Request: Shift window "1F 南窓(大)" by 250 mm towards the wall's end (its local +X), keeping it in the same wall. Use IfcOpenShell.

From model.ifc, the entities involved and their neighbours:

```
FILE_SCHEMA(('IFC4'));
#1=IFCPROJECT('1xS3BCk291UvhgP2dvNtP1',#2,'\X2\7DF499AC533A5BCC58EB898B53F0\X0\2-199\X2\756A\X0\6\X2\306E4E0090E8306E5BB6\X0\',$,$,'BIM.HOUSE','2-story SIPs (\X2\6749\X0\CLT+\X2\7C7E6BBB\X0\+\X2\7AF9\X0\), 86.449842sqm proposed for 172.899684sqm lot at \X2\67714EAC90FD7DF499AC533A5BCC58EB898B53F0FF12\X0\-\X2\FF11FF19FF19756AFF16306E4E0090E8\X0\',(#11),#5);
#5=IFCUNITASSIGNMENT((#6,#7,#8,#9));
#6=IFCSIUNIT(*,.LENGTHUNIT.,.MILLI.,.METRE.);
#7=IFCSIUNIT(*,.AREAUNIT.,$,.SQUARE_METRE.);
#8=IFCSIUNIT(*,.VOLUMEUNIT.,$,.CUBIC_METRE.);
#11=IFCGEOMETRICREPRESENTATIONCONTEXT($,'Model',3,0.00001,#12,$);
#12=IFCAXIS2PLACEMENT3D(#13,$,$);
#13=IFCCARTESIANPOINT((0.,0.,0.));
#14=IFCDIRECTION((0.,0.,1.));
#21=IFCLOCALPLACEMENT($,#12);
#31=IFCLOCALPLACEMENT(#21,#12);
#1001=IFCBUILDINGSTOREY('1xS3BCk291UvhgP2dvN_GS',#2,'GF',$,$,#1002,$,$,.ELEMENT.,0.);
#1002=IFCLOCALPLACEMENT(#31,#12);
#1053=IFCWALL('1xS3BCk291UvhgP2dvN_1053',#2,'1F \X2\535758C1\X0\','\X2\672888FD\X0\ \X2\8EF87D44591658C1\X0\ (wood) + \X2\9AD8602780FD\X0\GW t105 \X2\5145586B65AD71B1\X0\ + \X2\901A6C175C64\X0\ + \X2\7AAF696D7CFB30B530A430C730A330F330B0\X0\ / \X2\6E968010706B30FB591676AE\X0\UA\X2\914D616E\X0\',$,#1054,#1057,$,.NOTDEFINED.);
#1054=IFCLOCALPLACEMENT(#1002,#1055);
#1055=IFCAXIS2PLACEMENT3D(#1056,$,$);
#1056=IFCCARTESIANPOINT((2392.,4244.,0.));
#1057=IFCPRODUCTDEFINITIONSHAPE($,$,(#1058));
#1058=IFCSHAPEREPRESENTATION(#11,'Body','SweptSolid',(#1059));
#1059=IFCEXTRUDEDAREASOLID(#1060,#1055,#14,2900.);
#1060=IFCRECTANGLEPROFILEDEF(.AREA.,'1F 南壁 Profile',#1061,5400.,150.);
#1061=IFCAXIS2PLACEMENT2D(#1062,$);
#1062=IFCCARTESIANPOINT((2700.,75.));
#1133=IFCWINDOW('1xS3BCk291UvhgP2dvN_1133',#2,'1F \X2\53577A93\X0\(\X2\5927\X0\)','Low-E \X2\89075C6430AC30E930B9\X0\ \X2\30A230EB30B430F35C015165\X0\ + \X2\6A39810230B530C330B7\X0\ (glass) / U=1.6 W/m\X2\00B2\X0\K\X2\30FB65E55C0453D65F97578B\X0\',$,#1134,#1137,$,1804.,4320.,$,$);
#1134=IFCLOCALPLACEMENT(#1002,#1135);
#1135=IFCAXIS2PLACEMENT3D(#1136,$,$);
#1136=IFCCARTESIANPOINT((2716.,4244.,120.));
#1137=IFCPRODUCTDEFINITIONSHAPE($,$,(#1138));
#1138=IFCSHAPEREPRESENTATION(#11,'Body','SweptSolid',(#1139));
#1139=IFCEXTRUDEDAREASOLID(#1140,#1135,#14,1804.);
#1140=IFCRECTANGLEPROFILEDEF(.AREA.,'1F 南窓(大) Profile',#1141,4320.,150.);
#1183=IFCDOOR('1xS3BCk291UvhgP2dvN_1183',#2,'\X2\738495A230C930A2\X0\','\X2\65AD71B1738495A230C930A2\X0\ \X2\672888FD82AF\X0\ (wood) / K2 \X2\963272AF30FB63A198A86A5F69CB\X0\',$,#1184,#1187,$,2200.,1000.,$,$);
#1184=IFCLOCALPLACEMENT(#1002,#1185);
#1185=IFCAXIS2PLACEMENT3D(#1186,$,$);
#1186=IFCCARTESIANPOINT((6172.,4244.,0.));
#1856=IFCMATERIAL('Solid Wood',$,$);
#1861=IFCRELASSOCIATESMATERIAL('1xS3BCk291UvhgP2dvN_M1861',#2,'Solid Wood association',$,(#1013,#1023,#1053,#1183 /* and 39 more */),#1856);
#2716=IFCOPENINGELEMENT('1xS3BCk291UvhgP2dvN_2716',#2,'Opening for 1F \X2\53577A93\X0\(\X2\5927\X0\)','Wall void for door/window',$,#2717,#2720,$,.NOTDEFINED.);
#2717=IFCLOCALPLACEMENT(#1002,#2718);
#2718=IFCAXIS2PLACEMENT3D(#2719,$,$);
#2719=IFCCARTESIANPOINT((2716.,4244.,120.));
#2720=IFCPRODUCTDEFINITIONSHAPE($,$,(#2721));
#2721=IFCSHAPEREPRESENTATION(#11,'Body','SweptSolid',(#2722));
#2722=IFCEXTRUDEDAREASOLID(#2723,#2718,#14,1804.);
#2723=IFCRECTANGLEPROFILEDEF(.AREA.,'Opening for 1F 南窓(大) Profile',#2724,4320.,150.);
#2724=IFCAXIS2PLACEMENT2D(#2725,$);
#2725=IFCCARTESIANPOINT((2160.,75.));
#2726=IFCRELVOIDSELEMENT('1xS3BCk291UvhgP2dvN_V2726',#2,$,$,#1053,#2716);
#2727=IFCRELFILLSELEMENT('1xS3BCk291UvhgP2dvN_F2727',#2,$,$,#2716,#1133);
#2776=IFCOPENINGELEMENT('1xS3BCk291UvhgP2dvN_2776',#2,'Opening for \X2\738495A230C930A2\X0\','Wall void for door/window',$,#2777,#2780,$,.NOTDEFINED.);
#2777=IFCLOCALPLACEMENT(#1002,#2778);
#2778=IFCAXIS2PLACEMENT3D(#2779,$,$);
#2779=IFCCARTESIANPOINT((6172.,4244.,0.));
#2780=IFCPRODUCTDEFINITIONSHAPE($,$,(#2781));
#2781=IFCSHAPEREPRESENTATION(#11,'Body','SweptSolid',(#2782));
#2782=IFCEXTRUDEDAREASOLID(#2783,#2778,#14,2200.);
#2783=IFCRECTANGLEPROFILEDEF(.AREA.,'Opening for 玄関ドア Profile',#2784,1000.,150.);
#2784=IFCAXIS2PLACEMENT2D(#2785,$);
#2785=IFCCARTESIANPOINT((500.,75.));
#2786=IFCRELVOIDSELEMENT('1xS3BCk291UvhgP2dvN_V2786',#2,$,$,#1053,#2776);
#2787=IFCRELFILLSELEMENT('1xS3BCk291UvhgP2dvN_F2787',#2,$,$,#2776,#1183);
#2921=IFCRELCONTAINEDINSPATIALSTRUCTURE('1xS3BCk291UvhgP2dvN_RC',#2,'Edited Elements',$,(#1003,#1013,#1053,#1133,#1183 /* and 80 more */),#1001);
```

```python
import ifcopenshell
import ifcopenshell.api.geometry
import ifcopenshell.util.placement
import ifcopenshell.util.unit

model = ifcopenshell.open("model.ifc")
unit_scale = ifcopenshell.util.unit.calculate_unit_scale(model)

window = model.by_guid("1xS3BCk291UvhgP2dvN_1133")
opening = window.FillsVoids[0].RelatingOpeningElement
wall = opening.VoidsElements[0].RelatingBuildingElement

wall_matrix = ifcopenshell.util.placement.get_local_placement(wall.ObjectPlacement)
shift = wall_matrix[:3, 0] * 0.25 / unit_scale
before = ifcopenshell.util.placement.get_local_placement(window.ObjectPlacement)[:3, 3].copy()

# The window is not placed relative to its opening, so move both.
for product in (opening, window):
    matrix = ifcopenshell.util.placement.get_local_placement(product.ObjectPlacement)
    matrix[:3, 3] += shift
    ifcopenshell.api.geometry.edit_object_placement(model, product=product, matrix=matrix, is_si=False)

after = ifcopenshell.util.placement.get_local_placement(window.ObjectPlacement)[:3, 3]
print("window moved by", (after - before).round(3) + 0.0)

model.write("model_v2.ifc")
```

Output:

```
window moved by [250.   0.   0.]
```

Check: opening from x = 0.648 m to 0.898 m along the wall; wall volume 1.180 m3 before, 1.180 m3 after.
